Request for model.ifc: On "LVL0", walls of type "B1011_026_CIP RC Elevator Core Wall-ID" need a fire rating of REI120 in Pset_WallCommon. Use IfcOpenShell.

First a look at what the model holds.

```python
import ifcopenshell
import ifcopenshell.util.element

model = ifcopenshell.open("model.ifc")
print(model.schema)
storey = next(s for s in model.by_type("IfcBuildingStorey") if s.Name == "LVL0")
walls = [e for e in ifcopenshell.util.element.get_decomposition(storey) if e.is_a("IfcWall")]
seen = {}
for e in walls:
    element_type = ifcopenshell.util.element.get_type(e)
    key = (element_type.Name if element_type != e and element_type else None, ifcopenshell.util.element.get_pset(e, "Pset_WallCommon", "FireRating"))
    seen[key] = seen.get(key, 0) + 1
for (name, value), count in sorted(seen.items(), key=str):
    print(count, "x", name, "|", value)
```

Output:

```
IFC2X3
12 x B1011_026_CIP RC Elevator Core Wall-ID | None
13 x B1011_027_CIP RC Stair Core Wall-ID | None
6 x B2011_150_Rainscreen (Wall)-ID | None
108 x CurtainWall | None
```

```python
import ifcopenshell
import ifcopenshell.api.pset
import ifcopenshell.util.element

model = ifcopenshell.open("model.ifc")

storey = next(s for s in model.by_type("IfcBuildingStorey") if s.Name == "LVL0")
walls = [e for e in ifcopenshell.util.element.get_decomposition(storey) if e.is_a("IfcWall")]

count = 0
for e in walls:
    element_type = ifcopenshell.util.element.get_type(e)
    if element_type in (None, e) or element_type.Name != "B1011_026_CIP RC Elevator Core Wall-ID":
        continue
    found = ifcopenshell.util.element.get_pset(e, "Pset_WallCommon", should_inherit=False)
    if found:
        pset = model.by_id(found["id"])
        if len(ifcopenshell.util.element.get_elements_by_pset(pset)) > 1:
            pset = ifcopenshell.api.pset.unshare_pset(model, products=[e], pset=pset)[0]
    else:
        pset = ifcopenshell.api.pset.add_pset(model, product=e, name="Pset_WallCommon")
    ifcopenshell.api.pset.edit_pset(model, pset=pset, properties={"FireRating": "REI120"})
    count += 1

print(count, "walls updated")

model.write("model_v2.ifc")
```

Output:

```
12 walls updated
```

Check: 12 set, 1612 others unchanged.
